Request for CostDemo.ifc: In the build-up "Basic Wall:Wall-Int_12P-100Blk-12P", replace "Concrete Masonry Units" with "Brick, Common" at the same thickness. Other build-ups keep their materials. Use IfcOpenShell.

First a look at what the model holds.

```python
import ifcopenshell
import ifcopenshell.util.element

model = ifcopenshell.open("CostDemo.ifc")
print(model.schema)
for layer_set in model.by_type("IfcMaterialLayerSet"):
    if layer_set.LayerSetName == "Basic Wall:Wall-Int_12P-100Blk-12P":
        for layer in layer_set.MaterialLayers:
            print(layer.id(), layer.Material and layer.Material.Name, layer.LayerThickness, sep=" | ")
        print(len(ifcopenshell.util.element.get_elements_by_material(model, layer_set)), "elements and types use it")
print(sorted(m.Name for m in model.by_type("IfcMaterial") if m.Name)[:60])
```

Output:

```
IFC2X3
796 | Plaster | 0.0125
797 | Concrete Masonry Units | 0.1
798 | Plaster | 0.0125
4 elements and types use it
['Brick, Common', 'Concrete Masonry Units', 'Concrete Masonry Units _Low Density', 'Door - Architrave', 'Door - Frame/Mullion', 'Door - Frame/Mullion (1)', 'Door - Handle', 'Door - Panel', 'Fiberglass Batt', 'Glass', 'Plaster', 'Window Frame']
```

```python
import ifcopenshell
import ifcopenshell.api.material

model = ifcopenshell.open("CostDemo.ifc")

layer_set = next(s for s in model.by_type("IfcMaterialLayerSet") if s.LayerSetName == "Basic Wall:Wall-Int_12P-100Blk-12P")
layer = next(l for l in layer_set.MaterialLayers if l.Material and l.Material.Name == "Concrete Masonry Units")
material = next(m for m in model.by_type("IfcMaterial") if m.Name == "Brick, Common")

# Point this one layer at the other material; renaming the old one would change it everywhere.
ifcopenshell.api.material.edit_layer(model, layer=layer, attributes={}, material=material)

print([l.Material.Name if l.Material else None for l in layer_set.MaterialLayers])

model.write("CostDemo_edited.ifc")
```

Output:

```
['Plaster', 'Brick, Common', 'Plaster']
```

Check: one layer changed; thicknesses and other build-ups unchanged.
